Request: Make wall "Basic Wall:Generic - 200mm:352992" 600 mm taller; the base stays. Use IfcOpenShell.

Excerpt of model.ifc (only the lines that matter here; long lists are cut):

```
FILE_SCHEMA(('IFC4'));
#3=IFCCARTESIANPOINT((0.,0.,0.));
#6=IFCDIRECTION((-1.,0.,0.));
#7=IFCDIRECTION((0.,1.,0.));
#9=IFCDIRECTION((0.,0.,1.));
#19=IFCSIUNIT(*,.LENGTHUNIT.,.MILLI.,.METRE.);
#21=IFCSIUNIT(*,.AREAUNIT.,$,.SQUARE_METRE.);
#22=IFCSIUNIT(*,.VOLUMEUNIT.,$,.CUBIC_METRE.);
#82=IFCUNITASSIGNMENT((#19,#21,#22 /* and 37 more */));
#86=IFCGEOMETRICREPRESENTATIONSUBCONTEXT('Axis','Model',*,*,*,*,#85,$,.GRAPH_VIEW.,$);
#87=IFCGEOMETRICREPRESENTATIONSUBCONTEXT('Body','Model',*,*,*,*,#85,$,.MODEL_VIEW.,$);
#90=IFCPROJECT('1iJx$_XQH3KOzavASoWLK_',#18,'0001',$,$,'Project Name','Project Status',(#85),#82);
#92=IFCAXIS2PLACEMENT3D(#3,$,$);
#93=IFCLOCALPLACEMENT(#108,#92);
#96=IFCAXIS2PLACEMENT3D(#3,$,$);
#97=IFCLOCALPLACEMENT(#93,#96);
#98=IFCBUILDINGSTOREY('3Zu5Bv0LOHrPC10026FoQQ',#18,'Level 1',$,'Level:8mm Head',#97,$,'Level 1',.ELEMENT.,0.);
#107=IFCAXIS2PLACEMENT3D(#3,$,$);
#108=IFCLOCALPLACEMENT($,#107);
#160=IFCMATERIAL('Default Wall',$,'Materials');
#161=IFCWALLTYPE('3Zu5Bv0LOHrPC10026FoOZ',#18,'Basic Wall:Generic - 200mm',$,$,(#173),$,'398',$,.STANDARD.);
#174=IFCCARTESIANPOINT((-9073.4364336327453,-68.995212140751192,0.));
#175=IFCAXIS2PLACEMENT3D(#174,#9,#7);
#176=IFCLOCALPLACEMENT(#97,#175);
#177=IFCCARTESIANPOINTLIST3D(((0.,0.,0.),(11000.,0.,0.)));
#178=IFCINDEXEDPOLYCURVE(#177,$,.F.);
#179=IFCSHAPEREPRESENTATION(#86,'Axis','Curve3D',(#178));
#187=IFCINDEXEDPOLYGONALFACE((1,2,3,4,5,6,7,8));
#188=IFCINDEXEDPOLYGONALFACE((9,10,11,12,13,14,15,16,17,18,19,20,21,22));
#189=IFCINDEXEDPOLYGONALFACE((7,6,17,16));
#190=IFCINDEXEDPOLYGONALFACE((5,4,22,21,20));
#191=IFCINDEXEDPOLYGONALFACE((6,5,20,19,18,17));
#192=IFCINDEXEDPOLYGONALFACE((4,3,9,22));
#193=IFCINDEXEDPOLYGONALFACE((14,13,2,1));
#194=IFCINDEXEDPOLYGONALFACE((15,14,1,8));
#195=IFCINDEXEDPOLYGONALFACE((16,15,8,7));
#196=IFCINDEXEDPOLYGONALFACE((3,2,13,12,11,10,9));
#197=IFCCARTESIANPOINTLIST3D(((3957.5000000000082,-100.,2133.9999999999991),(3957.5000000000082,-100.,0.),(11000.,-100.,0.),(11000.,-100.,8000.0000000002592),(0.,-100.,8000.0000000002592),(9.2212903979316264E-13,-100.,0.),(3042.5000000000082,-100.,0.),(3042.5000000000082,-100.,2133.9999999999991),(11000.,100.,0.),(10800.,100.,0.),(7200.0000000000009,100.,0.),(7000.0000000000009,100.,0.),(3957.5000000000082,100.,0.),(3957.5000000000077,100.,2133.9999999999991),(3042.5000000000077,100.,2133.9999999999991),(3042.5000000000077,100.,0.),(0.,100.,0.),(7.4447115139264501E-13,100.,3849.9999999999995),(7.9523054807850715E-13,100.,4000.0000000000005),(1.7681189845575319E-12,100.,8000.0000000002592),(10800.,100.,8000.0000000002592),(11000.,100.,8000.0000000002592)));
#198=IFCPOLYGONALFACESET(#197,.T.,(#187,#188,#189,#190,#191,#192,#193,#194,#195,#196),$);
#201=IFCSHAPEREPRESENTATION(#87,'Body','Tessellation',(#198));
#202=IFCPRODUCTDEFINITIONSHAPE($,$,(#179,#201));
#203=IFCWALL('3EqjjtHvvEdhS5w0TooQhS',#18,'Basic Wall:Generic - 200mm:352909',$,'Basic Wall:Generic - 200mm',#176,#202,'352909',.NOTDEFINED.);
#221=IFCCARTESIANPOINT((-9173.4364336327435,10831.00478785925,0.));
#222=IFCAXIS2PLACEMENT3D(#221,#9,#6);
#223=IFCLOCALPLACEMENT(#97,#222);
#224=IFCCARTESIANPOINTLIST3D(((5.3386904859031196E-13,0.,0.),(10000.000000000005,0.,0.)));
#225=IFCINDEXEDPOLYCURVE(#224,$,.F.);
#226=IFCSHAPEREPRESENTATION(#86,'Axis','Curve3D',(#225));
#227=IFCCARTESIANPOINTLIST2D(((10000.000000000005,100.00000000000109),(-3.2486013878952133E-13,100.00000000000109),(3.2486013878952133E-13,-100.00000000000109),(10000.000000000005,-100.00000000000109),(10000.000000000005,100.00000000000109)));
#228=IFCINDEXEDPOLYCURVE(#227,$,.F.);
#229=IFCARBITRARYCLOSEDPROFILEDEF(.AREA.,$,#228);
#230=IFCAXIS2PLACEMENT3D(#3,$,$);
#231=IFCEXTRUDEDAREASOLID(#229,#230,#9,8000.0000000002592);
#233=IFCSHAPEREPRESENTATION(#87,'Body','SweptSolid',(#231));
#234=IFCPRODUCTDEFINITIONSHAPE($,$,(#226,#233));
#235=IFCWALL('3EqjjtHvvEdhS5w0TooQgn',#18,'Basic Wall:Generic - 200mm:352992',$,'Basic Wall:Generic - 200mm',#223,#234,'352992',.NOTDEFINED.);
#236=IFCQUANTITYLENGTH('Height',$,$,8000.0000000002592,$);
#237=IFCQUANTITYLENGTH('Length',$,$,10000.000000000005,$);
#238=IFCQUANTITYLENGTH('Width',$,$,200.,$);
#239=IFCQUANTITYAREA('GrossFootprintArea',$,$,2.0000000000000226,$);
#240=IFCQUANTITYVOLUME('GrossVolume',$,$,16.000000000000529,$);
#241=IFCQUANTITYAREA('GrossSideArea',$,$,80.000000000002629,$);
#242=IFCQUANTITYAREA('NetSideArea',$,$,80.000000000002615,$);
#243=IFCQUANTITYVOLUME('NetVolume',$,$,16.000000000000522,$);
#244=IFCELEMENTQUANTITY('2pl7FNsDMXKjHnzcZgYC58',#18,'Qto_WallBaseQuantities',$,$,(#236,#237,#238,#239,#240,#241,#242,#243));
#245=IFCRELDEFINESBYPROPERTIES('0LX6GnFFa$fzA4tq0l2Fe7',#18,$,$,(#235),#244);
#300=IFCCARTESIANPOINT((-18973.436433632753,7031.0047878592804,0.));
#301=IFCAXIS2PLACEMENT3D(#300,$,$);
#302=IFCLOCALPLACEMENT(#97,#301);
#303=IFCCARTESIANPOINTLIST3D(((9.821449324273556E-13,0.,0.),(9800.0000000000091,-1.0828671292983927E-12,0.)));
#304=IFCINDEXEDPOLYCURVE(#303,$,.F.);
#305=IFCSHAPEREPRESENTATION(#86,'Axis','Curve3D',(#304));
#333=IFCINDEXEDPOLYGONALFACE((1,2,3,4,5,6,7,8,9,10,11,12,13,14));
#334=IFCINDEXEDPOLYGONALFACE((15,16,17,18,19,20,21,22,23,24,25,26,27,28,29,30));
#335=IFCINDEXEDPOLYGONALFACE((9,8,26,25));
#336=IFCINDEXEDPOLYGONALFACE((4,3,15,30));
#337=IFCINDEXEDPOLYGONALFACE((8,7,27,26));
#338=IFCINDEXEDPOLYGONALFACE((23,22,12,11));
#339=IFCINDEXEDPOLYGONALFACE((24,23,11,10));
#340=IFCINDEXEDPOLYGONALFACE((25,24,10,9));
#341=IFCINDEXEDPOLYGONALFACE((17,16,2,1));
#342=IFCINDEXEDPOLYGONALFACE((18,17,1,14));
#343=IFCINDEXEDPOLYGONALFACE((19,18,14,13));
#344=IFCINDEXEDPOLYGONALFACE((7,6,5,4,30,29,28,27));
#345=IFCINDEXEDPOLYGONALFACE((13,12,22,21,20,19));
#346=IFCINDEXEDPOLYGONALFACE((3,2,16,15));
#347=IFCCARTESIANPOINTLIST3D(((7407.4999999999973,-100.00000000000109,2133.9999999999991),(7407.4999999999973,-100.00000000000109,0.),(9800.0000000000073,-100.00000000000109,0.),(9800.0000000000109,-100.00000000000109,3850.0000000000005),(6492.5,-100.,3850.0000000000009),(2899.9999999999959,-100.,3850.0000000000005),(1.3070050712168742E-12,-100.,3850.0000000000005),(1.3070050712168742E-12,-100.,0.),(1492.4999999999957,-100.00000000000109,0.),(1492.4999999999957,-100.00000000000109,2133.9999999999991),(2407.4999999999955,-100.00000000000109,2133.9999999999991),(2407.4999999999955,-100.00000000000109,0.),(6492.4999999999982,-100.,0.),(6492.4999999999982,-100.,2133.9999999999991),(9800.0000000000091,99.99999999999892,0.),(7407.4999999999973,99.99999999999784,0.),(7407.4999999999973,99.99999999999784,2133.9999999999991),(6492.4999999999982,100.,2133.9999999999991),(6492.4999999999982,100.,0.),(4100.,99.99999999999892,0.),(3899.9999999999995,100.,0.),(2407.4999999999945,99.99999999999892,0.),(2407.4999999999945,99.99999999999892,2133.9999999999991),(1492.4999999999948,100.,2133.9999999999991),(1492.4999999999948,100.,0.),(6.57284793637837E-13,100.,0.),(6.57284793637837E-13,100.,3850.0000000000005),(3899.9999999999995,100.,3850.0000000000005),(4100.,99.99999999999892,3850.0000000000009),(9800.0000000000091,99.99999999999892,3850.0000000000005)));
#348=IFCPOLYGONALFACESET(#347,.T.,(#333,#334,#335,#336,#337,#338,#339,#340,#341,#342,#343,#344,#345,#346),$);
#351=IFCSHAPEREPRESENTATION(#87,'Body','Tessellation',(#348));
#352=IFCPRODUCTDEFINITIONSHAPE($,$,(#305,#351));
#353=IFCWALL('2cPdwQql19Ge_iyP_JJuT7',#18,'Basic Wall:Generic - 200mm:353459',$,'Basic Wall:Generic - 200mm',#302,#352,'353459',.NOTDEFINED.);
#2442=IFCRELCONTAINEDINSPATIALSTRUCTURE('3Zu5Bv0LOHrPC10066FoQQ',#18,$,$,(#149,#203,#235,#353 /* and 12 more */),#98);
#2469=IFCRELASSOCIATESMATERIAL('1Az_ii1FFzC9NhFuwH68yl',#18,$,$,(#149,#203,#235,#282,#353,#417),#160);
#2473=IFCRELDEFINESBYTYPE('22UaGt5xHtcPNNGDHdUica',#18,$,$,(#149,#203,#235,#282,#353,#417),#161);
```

```python
import ifcopenshell
import ifcopenshell.api.pset
import ifcopenshell.geom
import ifcopenshell.util.element
import ifcopenshell.util.representation
import ifcopenshell.util.shape
import ifcopenshell.util.unit

model = ifcopenshell.open("model.ifc")
unit_scale = ifcopenshell.util.unit.calculate_unit_scale(model)
area_scale = ifcopenshell.util.unit.calculate_unit_scale(model, "AREAUNIT")
volume_scale = ifcopenshell.util.unit.calculate_unit_scale(model, "VOLUMEUNIT")
settings = ifcopenshell.geom.settings()


def volume(element):
    """Net volume in cubic metres, openings subtracted."""
    shape = ifcopenshell.geom.create_shape(settings, element)
    return ifcopenshell.util.shape.get_volume(shape.geometry)


wall = model.by_id(235)
before = volume(wall)

body = ifcopenshell.util.representation.get_representation(wall, "Model", "Body")
solid = body.Items[0]
old_height = solid.Depth
solid.Depth += 600.0
after = volume(wall)
thickness = 0.2  # wall thickness in metres

# Update the stored height, areas and volumes.
qto = model.by_id(ifcopenshell.util.element.get_pset(wall, "Qto_WallBaseQuantities", should_inherit=False)["id"])
ifcopenshell.api.pset.edit_qto(model, qto=qto, properties={
    "Height": solid.Depth,
    "GrossVolume": ifcopenshell.util.element.get_pset(wall, "Qto_WallBaseQuantities", "GrossVolume") * solid.Depth / old_height,
    "GrossSideArea": ifcopenshell.util.element.get_pset(wall, "Qto_WallBaseQuantities", "GrossSideArea") * solid.Depth / old_height,
    "NetSideArea": after / thickness / area_scale,
    "NetVolume": after / volume_scale,
})

print(f"height {old_height:g} -> {solid.Depth:g}, volume {before:.3f} -> {after:.3f} m3")

model.write("model-out.ifc")
```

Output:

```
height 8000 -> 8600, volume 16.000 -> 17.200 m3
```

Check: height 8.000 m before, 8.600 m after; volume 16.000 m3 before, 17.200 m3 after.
